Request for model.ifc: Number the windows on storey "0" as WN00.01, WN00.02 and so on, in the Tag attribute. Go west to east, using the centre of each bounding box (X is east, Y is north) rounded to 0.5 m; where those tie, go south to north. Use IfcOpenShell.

First a look at what the model holds.

```python
import ifcopenshell
import ifcopenshell.util.element
import ifcopenshell.util.placement

model = ifcopenshell.open("model.ifc")
print(model.schema)
storey = next(s for s in model.by_type("IfcBuildingStorey") if s.Name == "0")
windows = [e for e in ifcopenshell.util.element.get_decomposition(storey) if e.is_a("IfcWindow")]
for e in sorted(windows, key=lambda e: e.id()):
    origin = ifcopenshell.util.placement.get_local_placement(e.ObjectPlacement)[:3, 3]
    print(e.id(), e.Tag, e.Name, origin.round(2) + 0.0, sep=" | ")
```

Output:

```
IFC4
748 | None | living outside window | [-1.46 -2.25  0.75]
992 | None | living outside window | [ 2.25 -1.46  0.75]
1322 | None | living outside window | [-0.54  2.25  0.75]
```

```python
import ifcopenshell
import ifcopenshell.geom
import ifcopenshell.util.element
import ifcopenshell.util.shape

model = ifcopenshell.open("model.ifc")
settings = ifcopenshell.geom.settings()
settings.set("use-world-coords", True)


def centre(element):
    shape = ifcopenshell.geom.create_shape(settings, element)
    return ifcopenshell.util.shape.get_bbox_centroid(shape.geometry)


storey = next(s for s in model.by_type("IfcBuildingStorey") if s.Name == "0")
windows = [e for e in ifcopenshell.util.element.get_decomposition(storey) if e.is_a("IfcWindow")]

# Insertion points can sit at a corner or the storey origin, so sort by the geometry (in metres).
centres = {e: centre(e) for e in windows}
windows.sort(key=lambda e: (round(centres[e][0] / 0.5), centres[e][1]))

for i, e in enumerate(windows, start=1):
    number = f"WN00.{i:02d}"
    e.Tag = number
    print(e.id(), number)

model.write("model-out.ifc")
```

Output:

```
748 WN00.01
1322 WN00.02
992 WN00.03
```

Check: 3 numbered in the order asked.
